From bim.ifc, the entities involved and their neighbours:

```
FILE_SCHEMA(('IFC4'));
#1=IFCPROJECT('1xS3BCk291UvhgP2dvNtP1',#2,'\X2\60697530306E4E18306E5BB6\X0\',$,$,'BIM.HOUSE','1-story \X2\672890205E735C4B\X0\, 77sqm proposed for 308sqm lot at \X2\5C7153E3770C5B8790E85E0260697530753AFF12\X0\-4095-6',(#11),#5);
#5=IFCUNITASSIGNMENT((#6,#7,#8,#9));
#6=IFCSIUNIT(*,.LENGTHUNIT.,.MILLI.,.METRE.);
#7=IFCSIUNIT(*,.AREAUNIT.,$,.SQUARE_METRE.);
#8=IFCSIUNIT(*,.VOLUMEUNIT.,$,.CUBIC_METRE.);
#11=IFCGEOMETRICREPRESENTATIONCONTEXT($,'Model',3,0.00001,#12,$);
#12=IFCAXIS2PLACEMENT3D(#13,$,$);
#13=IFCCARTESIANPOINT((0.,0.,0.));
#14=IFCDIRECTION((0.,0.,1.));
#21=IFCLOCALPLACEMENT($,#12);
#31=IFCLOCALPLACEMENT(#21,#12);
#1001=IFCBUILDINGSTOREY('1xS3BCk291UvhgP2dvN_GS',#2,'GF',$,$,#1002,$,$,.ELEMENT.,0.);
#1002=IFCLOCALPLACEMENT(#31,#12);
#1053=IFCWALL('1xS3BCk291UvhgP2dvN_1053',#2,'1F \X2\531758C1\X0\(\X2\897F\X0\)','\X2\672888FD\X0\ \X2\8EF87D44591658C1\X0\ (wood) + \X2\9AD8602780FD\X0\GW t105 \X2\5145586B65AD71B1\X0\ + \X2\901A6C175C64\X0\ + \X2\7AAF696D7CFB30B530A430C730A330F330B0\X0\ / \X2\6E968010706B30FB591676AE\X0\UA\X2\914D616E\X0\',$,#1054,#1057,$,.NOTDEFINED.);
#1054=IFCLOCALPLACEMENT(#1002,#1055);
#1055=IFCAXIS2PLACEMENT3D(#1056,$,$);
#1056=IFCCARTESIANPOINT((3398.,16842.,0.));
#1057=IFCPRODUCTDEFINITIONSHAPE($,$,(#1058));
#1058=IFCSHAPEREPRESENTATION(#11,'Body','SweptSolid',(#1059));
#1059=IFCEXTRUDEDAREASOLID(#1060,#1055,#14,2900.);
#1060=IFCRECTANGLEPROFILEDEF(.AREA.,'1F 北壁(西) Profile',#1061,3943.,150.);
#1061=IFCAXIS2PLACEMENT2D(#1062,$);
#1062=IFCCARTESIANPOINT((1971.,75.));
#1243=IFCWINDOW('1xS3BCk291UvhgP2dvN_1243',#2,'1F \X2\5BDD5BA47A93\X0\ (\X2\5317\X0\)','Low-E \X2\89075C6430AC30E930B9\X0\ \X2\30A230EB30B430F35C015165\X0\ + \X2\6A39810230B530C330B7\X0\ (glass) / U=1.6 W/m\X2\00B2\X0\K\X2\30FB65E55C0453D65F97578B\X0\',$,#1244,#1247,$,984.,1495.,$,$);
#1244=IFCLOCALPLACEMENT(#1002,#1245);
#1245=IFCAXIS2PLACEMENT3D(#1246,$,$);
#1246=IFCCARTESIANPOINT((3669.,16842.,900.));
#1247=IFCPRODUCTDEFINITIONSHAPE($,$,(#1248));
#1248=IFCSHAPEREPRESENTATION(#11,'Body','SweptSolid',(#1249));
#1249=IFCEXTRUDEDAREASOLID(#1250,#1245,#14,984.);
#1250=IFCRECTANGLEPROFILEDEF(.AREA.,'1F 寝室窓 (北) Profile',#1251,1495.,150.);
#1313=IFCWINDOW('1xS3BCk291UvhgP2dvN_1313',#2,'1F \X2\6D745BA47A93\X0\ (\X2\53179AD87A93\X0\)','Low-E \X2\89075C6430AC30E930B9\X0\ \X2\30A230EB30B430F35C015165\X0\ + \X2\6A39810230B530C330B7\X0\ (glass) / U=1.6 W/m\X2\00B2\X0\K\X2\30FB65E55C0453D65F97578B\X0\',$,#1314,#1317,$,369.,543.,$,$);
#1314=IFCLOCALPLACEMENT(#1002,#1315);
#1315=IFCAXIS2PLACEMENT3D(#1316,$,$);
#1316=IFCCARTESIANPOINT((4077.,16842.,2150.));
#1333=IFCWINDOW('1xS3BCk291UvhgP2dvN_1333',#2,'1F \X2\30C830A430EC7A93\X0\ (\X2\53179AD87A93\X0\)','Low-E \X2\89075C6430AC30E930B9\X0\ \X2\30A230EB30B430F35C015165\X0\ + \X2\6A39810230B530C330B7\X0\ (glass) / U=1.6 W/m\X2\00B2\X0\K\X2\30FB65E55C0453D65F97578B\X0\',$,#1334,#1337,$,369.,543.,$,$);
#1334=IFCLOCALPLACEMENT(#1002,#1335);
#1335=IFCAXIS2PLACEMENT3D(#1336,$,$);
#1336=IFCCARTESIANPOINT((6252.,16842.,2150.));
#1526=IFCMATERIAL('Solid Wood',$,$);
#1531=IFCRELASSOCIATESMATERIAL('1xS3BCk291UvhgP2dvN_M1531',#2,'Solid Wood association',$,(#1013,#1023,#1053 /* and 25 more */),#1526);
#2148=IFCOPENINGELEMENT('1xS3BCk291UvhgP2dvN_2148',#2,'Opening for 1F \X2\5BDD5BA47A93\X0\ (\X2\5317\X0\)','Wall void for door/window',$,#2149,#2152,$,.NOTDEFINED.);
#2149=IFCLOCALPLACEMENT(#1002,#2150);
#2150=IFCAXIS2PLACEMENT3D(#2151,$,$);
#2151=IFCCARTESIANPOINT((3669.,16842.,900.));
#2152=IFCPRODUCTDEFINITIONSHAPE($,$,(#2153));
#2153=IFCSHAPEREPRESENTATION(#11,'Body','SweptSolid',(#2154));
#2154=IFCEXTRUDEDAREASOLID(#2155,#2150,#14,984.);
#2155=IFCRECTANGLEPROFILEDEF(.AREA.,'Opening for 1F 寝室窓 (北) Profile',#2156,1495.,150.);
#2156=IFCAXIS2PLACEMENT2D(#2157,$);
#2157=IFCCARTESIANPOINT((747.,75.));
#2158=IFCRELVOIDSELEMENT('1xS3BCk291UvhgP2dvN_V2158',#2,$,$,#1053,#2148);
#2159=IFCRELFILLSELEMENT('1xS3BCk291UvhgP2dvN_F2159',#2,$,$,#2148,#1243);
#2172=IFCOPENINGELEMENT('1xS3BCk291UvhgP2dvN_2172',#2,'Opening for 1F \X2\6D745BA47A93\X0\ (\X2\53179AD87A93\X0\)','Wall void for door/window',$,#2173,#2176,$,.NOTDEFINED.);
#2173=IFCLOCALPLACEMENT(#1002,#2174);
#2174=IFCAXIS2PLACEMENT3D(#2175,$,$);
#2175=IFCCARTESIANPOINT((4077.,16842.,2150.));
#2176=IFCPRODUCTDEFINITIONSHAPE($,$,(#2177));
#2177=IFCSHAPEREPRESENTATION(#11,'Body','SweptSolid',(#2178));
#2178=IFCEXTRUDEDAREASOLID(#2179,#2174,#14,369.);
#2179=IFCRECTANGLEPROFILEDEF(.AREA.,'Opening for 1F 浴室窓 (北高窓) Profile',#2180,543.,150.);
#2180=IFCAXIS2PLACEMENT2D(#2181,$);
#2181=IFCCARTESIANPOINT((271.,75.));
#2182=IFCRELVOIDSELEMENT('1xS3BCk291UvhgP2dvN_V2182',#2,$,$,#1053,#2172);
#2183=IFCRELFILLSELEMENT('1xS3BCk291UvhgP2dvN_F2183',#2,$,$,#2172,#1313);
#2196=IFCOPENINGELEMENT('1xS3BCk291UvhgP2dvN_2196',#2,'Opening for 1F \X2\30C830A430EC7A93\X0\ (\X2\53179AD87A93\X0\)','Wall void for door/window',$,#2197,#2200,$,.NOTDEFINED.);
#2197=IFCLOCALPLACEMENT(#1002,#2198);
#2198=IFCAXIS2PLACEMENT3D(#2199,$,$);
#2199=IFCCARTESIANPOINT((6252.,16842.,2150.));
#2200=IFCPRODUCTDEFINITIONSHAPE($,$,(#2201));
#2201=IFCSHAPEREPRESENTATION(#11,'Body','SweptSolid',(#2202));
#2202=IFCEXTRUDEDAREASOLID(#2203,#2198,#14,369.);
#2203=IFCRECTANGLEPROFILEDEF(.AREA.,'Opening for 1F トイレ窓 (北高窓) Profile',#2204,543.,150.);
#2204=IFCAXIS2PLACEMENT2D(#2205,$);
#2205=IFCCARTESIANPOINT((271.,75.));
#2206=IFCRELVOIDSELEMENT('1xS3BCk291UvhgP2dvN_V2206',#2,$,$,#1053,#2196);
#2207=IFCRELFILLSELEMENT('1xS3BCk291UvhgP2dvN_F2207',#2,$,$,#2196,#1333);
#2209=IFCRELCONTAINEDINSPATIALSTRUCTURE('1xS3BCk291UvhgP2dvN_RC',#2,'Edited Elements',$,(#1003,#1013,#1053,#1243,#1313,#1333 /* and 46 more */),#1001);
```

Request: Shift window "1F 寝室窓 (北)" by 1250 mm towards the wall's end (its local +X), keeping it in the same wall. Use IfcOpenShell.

```python
import ifcopenshell
import ifcopenshell.api.geometry
import ifcopenshell.util.placement

model = ifcopenshell.open("bim.ifc")

window = model.by_guid("1xS3BCk291UvhgP2dvN_1243")
opening = window.FillsVoids[0].RelatingOpeningElement
wall = opening.VoidsElements[0].RelatingBuildingElement

wall_matrix = ifcopenshell.util.placement.get_local_placement(wall.ObjectPlacement)
shift = wall_matrix[:3, 0] * 1250.0
before = ifcopenshell.util.placement.get_local_placement(window.ObjectPlacement)[:3, 3].copy()

# The window is not placed relative to its opening, so move both.
for product in (opening, window):
    matrix = ifcopenshell.util.placement.get_local_placement(product.ObjectPlacement)
    matrix[:3, 3] += shift
    ifcopenshell.api.geometry.edit_object_placement(model, product=product, matrix=matrix, is_si=False)

after = ifcopenshell.util.placement.get_local_placement(window.ObjectPlacement)[:3, 3]
print("window moved by", (after - before).round(3) + 0.0)

model.write("bim_updated.ifc")
```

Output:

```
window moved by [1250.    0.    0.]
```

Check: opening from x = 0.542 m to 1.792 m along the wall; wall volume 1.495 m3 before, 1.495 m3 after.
